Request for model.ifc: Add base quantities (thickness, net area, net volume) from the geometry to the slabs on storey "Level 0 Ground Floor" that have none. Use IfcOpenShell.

First a look at what the model holds.

```python
import ifcopenshell
import ifcopenshell.util.element
import ifcopenshell.util.unit

model = ifcopenshell.open("model.ifc")
print(model.schema)
for unit_type in ("LENGTHUNIT", "AREAUNIT", "VOLUMEUNIT"):
    print(unit_type, ifcopenshell.util.unit.calculate_unit_scale(model, unit_type))
storey = next(s for s in model.by_type("IfcBuildingStorey") if s.Name == "Level 0 Ground Floor")
slabs = [e for e in ifcopenshell.util.element.get_decomposition(storey) if e.is_a("IfcSlab")]
for e in sorted(slabs, key=lambda e: e.id()):
    print(e.id(), e.is_a(), e.Name, list(ifcopenshell.util.element.get_psets(e, qtos_only=True)), sep=" | ")
```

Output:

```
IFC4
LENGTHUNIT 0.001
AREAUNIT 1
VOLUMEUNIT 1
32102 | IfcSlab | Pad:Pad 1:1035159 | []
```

```python
import ifcopenshell
import ifcopenshell.api.pset
import ifcopenshell.geom
import ifcopenshell.util.element
import ifcopenshell.util.shape
import ifcopenshell.util.unit

model = ifcopenshell.open("model.ifc")
unit_scale = ifcopenshell.util.unit.calculate_unit_scale(model)
area_scale = ifcopenshell.util.unit.calculate_unit_scale(model, "AREAUNIT")
volume_scale = ifcopenshell.util.unit.calculate_unit_scale(model, "VOLUMEUNIT")
settings = ifcopenshell.geom.settings()

storey = next(s for s in model.by_type("IfcBuildingStorey") if s.Name == "Level 0 Ground Floor")
slabs = [e for e in ifcopenshell.util.element.get_decomposition(storey) if e.is_a("IfcSlab")]

for e in sorted(slabs, key=lambda e: e.id()):
    if ifcopenshell.util.element.get_psets(e, qtos_only=True, should_inherit=False):
        continue
    # Geometry comes back in metres, in the element's own axes.
    shape = ifcopenshell.geom.create_shape(settings, e)
    values = {
        "Width": ifcopenshell.util.shape.get_z(shape.geometry) / unit_scale,
        "NetArea": ifcopenshell.util.shape.get_footprint_area(shape.geometry) / area_scale,
        "NetVolume": ifcopenshell.util.shape.get_volume(shape.geometry) / volume_scale,
    }
    qto = ifcopenshell.api.pset.add_qto(model, product=e, name="Qto_SlabBaseQuantities")
    ifcopenshell.api.pset.edit_qto(model, qto=qto, properties=values)
    print(e.id(), {k: round(v, 3) for k, v in values.items()})

model.write("model_v2.ifc")
```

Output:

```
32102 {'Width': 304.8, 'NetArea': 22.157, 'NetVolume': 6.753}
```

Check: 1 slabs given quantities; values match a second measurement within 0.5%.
